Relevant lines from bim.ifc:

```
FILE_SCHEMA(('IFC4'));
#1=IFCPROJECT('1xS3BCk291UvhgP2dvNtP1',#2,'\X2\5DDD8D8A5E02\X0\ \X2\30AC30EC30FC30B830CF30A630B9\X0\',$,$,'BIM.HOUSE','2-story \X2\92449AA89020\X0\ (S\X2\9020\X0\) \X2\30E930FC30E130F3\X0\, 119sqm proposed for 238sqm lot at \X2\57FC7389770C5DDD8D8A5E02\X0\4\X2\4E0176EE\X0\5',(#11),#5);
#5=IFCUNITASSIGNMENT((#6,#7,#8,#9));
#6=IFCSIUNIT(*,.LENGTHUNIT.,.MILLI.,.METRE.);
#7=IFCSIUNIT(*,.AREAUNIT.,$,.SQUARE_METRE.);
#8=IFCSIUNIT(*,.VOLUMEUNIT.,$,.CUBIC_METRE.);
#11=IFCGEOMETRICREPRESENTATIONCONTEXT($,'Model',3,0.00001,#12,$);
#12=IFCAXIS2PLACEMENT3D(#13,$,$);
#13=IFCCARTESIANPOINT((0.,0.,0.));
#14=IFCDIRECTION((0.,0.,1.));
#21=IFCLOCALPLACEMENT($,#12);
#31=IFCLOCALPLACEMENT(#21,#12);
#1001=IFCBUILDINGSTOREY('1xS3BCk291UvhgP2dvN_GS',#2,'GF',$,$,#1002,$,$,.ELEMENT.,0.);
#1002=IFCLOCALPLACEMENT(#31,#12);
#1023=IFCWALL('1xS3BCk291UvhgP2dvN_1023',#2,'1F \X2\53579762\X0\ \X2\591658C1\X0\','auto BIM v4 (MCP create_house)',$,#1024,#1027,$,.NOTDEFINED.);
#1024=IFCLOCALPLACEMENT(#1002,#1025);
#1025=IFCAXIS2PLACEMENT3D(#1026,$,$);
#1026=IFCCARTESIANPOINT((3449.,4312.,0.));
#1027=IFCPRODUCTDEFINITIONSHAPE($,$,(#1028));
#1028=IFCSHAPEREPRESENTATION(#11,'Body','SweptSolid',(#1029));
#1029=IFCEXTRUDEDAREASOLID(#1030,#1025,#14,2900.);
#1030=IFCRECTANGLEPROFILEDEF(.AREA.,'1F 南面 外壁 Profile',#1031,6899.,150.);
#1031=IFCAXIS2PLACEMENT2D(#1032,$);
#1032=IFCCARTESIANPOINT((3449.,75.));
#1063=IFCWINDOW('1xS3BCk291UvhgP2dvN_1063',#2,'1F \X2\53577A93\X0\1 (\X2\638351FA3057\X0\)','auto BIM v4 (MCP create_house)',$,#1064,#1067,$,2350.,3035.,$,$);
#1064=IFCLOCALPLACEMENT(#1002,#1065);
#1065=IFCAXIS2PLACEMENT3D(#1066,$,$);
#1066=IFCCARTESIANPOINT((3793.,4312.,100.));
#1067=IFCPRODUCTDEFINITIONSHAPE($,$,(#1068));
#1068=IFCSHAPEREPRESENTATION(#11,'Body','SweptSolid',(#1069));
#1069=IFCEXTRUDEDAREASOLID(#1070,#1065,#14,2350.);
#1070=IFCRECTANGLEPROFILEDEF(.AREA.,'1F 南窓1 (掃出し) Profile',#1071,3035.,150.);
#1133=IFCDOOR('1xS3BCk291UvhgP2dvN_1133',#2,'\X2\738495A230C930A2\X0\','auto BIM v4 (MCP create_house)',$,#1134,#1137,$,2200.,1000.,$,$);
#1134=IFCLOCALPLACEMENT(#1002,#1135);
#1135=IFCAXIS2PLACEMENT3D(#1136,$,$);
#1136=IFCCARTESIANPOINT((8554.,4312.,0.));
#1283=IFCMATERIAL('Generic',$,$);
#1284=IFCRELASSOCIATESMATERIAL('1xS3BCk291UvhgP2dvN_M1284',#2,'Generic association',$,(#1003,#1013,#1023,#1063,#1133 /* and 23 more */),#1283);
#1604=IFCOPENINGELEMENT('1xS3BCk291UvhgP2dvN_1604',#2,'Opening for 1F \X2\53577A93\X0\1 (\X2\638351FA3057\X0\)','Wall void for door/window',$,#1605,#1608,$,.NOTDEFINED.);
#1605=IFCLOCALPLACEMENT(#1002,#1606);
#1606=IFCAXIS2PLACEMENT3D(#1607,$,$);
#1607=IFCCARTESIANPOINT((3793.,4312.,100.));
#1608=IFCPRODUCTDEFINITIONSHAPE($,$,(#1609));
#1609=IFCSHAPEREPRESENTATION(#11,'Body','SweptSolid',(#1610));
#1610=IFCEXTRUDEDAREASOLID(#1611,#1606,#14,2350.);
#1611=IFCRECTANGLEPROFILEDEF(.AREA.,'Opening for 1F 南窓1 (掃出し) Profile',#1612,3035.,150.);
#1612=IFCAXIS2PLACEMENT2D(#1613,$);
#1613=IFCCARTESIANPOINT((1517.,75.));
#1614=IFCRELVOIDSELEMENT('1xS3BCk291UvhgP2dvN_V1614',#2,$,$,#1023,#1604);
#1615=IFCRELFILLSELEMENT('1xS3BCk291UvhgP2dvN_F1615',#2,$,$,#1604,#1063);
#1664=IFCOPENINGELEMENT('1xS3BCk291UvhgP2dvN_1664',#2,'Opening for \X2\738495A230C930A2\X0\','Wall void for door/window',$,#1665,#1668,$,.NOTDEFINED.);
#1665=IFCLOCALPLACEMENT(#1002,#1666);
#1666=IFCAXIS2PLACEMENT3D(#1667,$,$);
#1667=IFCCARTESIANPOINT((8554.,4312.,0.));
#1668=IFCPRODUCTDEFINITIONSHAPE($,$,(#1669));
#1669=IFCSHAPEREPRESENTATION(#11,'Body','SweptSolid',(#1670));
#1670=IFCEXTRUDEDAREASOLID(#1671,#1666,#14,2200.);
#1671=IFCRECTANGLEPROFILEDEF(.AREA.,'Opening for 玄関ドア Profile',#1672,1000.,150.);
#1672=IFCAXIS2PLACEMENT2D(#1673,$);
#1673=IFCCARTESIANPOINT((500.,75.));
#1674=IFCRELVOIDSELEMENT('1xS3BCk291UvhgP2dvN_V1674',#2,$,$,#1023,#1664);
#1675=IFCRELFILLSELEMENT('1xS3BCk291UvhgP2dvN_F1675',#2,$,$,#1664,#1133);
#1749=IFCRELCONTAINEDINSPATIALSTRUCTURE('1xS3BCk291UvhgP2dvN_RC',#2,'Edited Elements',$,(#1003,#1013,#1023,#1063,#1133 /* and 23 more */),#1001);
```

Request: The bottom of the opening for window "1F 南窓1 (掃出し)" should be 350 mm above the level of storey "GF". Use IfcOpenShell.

```python
import numpy as np
import ifcopenshell
import ifcopenshell.api.geometry
import ifcopenshell.geom
import ifcopenshell.util.element
import ifcopenshell.util.placement
import ifcopenshell.util.shape
import ifcopenshell.util.unit

model = ifcopenshell.open("bim.ifc")
unit_scale = ifcopenshell.util.unit.calculate_unit_scale(model)

window = model.by_guid("1xS3BCk291UvhgP2dvN_1063")
opening = window.FillsVoids[0].RelatingOpeningElement
storey = ifcopenshell.util.element.get_container(window, ifc_class="IfcBuildingStorey")
level = ifcopenshell.util.placement.get_local_placement(storey.ObjectPlacement)[2, 3]

# The opening's origin need not be at the sill, so measure its lowest point.
shape = ifcopenshell.geom.create_shape(ifcopenshell.geom.settings(), opening)
bottom = ifcopenshell.util.shape.get_shape_bottom_elevation(shape, shape.geometry) / unit_scale
dz = level + 0.35 / unit_scale - bottom

shift = np.array([0.0, 0.0, dz])
# The window is not placed relative to its opening, so move both.
for product in (opening, window):
    matrix = ifcopenshell.util.placement.get_local_placement(product.ObjectPlacement)
    matrix[:3, 3] += shift
    ifcopenshell.api.geometry.edit_object_placement(model, product=product, matrix=matrix, is_si=False)

print(f"moved by {dz * unit_scale:+.3f} m")

model.write("bim_rev.ifc")
```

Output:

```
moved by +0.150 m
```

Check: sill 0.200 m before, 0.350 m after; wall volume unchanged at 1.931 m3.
